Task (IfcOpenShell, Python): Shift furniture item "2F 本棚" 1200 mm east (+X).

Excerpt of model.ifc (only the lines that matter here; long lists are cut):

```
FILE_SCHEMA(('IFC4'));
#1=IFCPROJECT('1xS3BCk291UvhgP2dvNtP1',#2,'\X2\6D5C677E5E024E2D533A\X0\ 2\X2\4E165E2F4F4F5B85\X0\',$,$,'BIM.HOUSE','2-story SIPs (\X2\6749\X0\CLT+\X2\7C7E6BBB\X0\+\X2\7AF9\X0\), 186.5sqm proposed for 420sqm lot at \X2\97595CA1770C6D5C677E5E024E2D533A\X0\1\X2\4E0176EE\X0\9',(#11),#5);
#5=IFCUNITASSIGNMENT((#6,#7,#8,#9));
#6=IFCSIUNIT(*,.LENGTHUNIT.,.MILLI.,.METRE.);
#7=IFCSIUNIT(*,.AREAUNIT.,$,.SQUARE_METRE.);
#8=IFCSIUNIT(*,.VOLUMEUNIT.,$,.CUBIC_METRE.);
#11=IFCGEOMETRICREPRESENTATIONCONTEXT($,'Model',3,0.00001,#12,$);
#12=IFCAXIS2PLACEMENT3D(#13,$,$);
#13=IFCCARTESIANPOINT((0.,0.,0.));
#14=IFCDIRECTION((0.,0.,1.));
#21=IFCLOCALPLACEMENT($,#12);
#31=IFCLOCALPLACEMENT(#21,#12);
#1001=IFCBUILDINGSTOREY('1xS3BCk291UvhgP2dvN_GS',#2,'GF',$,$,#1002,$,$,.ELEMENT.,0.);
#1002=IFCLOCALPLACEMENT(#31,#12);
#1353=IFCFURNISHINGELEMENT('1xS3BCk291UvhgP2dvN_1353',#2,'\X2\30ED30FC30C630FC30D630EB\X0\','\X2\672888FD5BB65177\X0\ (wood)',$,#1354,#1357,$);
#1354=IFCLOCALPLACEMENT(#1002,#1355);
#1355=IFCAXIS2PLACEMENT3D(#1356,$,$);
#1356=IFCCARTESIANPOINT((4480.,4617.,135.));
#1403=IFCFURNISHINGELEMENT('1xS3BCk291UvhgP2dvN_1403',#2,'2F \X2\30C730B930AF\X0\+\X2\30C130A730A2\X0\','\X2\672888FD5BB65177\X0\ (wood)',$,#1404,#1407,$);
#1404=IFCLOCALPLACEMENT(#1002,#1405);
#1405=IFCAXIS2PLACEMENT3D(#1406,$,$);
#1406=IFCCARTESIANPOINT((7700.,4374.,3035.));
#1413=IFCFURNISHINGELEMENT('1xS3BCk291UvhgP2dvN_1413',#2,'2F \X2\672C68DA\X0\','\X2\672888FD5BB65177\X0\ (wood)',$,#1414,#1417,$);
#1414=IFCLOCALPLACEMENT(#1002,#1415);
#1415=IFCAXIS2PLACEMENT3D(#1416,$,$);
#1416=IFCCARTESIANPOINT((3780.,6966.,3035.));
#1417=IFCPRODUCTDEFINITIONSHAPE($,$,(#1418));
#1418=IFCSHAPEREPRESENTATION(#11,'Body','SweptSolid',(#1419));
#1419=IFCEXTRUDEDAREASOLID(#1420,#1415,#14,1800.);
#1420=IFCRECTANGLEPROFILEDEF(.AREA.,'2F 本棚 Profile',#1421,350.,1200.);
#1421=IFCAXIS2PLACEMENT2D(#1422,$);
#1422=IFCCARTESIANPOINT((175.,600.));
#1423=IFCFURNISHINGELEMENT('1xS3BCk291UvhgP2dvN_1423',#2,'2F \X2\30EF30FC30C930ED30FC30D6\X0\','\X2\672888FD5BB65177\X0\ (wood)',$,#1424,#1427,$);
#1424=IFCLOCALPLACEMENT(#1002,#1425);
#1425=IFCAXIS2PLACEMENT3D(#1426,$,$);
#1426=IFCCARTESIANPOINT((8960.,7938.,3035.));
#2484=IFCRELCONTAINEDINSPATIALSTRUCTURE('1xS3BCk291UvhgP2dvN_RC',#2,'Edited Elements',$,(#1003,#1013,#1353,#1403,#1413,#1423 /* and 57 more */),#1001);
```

```python
import ifcopenshell
import ifcopenshell.api.geometry
import ifcopenshell.util.placement

model = ifcopenshell.open("model.ifc")

item = model.by_guid("1xS3BCk291UvhgP2dvN_1413")
matrix = ifcopenshell.util.placement.get_local_placement(item.ObjectPlacement)
matrix[0, 3] += 1200.0
ifcopenshell.api.geometry.edit_object_placement(model, product=item, matrix=matrix, is_si=False)

print(ifcopenshell.util.placement.get_local_placement(item.ObjectPlacement).round(3) + 0.0)

model.write("model_edited.ifc")
```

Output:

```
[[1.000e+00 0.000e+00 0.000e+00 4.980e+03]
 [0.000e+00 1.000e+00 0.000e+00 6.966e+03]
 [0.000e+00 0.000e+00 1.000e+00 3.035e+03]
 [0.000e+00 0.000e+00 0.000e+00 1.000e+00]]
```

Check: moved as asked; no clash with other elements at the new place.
